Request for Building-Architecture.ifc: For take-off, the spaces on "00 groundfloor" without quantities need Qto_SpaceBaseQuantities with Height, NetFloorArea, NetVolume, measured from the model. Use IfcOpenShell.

First a look at what the model holds.

```python
import ifcopenshell
import ifcopenshell.util.element
import ifcopenshell.util.unit

model = ifcopenshell.open("Building-Architecture.ifc")
print(model.schema)
for unit_type in ("LENGTHUNIT", "AREAUNIT", "VOLUMEUNIT"):
    print(unit_type, ifcopenshell.util.unit.calculate_unit_scale(model, unit_type))
storey = next(s for s in model.by_type("IfcBuildingStorey") if s.Name == "00 groundfloor")
spaces = [e for e in ifcopenshell.util.element.get_decomposition(storey) if e.is_a("IfcSpace")]
for e in sorted(spaces, key=lambda e: e.id()):
    print(e.id(), e.is_a(), e.Name, list(ifcopenshell.util.element.get_psets(e, qtos_only=True)), sep=" | ")
```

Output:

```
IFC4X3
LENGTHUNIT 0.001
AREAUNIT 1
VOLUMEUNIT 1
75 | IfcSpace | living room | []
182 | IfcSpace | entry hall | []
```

```python
import ifcopenshell
import ifcopenshell.api.pset
import ifcopenshell.geom
import ifcopenshell.util.element
import ifcopenshell.util.shape
import ifcopenshell.util.unit

model = ifcopenshell.open("Building-Architecture.ifc")
unit_scale = ifcopenshell.util.unit.calculate_unit_scale(model)
area_scale = ifcopenshell.util.unit.calculate_unit_scale(model, "AREAUNIT")
volume_scale = ifcopenshell.util.unit.calculate_unit_scale(model, "VOLUMEUNIT")
settings = ifcopenshell.geom.settings()

storey = next(s for s in model.by_type("IfcBuildingStorey") if s.Name == "00 groundfloor")
spaces = [e for e in ifcopenshell.util.element.get_decomposition(storey) if e.is_a("IfcSpace")]

for e in sorted(spaces, key=lambda e: e.id()):
    if ifcopenshell.util.element.get_psets(e, qtos_only=True, should_inherit=False):
        continue
    # Geometry comes back in metres, in the element's own axes.
    shape = ifcopenshell.geom.create_shape(settings, e)
    values = {
        "Height": ifcopenshell.util.shape.get_z(shape.geometry) / unit_scale,
        "NetFloorArea": ifcopenshell.util.shape.get_footprint_area(shape.geometry) / area_scale,
        "NetVolume": ifcopenshell.util.shape.get_volume(shape.geometry) / volume_scale,
    }
    qto = ifcopenshell.api.pset.add_qto(model, product=e, name="Qto_SpaceBaseQuantities")
    ifcopenshell.api.pset.edit_qto(model, qto=qto, properties=values)
    print(e.id(), {k: round(v, 3) for k, v in values.items()})

model.write("Building-Architecture_rev.ifc")
```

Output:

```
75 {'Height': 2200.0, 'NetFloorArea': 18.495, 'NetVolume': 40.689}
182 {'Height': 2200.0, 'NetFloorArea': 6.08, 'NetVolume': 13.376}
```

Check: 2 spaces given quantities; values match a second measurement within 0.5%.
